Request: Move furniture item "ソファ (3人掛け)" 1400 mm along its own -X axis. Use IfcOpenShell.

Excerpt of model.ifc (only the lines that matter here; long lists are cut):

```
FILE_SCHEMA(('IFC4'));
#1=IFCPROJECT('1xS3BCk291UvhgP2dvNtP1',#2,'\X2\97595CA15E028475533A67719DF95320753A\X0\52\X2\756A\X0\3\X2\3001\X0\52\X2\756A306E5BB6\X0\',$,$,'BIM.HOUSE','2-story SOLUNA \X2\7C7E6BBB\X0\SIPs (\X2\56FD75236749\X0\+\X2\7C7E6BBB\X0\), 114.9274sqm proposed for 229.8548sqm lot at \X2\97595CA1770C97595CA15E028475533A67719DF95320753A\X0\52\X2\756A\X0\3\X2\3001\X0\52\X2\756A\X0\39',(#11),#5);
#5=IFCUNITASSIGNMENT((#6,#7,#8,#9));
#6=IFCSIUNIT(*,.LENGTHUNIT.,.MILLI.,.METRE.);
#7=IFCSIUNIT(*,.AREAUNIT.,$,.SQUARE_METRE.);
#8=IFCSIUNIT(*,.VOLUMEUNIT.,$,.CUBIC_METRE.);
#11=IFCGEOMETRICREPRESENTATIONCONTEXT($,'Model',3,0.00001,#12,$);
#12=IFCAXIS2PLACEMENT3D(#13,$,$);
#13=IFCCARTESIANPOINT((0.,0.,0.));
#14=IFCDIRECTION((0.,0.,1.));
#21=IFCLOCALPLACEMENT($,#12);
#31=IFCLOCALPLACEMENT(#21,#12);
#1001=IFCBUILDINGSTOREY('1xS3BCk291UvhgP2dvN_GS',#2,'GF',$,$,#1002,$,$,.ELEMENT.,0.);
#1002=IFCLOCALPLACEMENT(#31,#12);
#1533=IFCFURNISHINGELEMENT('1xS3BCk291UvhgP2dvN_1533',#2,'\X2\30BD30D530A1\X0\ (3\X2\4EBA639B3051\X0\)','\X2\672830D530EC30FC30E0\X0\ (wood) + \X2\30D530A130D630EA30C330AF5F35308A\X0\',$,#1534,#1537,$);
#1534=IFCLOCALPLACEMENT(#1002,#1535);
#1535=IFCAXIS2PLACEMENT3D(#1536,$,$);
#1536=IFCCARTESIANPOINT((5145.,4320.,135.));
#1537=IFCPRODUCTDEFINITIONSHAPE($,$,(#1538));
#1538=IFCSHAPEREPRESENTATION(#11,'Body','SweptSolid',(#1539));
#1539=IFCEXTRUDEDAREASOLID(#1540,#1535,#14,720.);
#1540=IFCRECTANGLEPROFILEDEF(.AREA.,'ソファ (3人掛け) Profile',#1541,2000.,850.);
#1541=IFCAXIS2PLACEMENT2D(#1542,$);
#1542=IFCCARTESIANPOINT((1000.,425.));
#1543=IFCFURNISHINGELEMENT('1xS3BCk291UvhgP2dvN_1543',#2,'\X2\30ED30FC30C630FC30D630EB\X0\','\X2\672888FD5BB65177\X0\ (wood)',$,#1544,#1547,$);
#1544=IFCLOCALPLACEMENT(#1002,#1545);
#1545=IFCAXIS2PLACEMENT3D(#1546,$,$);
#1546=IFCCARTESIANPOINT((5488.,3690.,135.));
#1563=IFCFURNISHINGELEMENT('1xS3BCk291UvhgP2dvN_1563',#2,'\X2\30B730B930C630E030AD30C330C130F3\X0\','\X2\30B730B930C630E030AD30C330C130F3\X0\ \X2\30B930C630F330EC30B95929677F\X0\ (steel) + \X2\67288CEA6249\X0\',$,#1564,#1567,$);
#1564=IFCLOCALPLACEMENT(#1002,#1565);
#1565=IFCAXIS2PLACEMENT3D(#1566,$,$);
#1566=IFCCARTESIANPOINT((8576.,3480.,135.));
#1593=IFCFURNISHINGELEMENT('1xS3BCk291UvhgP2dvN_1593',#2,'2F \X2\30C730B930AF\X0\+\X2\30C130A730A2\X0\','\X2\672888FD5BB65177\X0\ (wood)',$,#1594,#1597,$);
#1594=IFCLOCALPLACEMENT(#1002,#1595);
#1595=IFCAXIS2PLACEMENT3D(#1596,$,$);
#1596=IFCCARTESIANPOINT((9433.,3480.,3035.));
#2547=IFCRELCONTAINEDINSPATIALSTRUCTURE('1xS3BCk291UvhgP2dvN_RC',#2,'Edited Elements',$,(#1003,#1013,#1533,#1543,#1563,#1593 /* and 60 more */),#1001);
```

```python
import ifcopenshell
import ifcopenshell.api.geometry
import ifcopenshell.util.placement

model = ifcopenshell.open("model.ifc")

item = model.by_guid("1xS3BCk291UvhgP2dvN_1533")
matrix = ifcopenshell.util.placement.get_local_placement(item.ObjectPlacement)
matrix[:3, 3] -= matrix[:3, 0] * 1400.0
ifcopenshell.api.geometry.edit_object_placement(model, product=item, matrix=matrix, is_si=False)

print(ifcopenshell.util.placement.get_local_placement(item.ObjectPlacement).round(3) + 0.0)

model.write("model_rev.ifc")
```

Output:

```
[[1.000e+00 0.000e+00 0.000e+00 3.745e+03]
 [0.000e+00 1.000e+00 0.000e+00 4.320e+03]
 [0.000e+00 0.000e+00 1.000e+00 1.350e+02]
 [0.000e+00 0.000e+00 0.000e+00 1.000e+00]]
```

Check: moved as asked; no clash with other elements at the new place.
